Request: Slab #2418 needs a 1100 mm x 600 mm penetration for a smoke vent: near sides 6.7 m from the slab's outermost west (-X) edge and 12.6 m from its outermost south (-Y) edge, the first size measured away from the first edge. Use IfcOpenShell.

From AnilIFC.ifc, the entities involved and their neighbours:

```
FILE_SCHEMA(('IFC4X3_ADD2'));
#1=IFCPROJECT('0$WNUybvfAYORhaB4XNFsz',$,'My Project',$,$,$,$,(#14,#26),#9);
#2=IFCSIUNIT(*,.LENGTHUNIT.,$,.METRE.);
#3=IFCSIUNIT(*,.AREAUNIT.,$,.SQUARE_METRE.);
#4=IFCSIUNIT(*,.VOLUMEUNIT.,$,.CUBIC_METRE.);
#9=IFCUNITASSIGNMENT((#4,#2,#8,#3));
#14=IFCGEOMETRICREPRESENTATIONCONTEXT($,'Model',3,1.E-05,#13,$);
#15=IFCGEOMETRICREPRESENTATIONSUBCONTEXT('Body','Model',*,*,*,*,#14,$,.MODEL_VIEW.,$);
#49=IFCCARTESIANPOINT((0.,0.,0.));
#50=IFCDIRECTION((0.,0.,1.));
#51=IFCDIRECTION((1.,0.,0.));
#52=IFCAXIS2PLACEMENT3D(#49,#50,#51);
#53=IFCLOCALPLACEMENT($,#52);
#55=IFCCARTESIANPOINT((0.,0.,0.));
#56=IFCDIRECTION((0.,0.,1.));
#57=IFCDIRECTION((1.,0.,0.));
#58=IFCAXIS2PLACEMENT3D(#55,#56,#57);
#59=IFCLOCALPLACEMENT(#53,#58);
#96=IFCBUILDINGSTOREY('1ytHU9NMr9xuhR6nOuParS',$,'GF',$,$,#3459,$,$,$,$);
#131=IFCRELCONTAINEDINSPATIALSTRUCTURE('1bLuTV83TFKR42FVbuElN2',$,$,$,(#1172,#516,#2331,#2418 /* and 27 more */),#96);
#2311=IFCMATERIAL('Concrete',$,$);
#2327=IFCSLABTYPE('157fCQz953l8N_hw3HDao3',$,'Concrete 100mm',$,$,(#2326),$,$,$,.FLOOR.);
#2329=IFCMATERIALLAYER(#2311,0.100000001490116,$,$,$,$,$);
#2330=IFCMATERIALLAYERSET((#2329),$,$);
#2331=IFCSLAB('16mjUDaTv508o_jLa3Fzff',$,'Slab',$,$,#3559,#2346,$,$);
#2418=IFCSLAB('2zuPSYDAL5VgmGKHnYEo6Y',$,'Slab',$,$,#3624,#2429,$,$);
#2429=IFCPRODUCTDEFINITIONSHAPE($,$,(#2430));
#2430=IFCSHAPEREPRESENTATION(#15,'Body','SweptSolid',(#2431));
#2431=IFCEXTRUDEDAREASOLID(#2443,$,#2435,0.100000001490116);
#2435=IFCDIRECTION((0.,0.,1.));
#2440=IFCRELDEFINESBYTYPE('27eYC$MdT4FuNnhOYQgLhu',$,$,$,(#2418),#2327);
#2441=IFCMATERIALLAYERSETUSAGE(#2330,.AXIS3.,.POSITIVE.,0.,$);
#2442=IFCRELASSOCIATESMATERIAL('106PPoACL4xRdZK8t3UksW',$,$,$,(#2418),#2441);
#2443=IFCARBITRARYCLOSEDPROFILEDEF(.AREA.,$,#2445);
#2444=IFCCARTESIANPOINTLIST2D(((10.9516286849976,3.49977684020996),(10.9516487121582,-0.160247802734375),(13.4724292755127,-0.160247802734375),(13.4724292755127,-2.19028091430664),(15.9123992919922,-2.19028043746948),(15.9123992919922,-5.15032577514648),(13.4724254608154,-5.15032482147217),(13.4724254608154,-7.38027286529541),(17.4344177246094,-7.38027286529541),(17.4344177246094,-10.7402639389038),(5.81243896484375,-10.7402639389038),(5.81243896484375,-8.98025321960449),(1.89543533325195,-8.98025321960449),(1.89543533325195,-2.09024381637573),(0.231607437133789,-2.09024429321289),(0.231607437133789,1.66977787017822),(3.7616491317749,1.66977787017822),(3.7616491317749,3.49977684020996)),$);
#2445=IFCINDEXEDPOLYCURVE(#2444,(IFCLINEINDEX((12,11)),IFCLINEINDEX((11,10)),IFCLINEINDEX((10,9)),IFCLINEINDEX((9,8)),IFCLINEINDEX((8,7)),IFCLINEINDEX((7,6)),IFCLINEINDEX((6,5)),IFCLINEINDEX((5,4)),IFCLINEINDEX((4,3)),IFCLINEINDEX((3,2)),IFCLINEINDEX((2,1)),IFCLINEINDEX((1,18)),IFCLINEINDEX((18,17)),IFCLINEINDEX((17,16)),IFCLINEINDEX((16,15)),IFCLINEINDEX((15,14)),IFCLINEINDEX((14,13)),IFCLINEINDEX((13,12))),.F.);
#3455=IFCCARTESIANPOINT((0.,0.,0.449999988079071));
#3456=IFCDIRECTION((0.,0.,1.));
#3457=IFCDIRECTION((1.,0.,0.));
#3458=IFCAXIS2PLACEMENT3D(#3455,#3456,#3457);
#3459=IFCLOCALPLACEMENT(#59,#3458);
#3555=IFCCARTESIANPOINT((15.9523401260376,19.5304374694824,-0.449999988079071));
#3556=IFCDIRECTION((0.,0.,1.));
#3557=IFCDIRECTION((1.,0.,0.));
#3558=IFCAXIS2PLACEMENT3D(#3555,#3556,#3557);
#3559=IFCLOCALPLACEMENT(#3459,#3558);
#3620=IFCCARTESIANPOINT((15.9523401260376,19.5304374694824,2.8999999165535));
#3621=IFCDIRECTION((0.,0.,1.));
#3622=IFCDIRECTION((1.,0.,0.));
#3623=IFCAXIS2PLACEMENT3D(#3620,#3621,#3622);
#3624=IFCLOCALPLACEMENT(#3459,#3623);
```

```python
import numpy as np
import ifcopenshell
import ifcopenshell.api.feature
import ifcopenshell.api.geometry
import ifcopenshell.api.root
import ifcopenshell.geom
import ifcopenshell.util.placement
import ifcopenshell.util.representation
import ifcopenshell.util.shape
import ifcopenshell.util.unit

model = ifcopenshell.open("AnilIFC.ifc")
unit_scale = ifcopenshell.util.unit.calculate_unit_scale(model)
settings = ifcopenshell.geom.settings()


def volume(element):
    """Net volume in cubic metres, openings subtracted."""
    shape = ifcopenshell.geom.create_shape(settings, element)
    return ifcopenshell.util.shape.get_volume(shape.geometry)


slab = model.by_guid("2zuPSYDAL5VgmGKHnYEo6Y")
before = volume(slab)

# Extent in the slab's own axes, in metres. The edges named are its -X and -Y sides.
slab_shape = ifcopenshell.geom.create_shape(settings, slab)
vertices = ifcopenshell.util.shape.get_vertices(slab_shape.geometry)
x_min, y_min, bottom = vertices.min(axis=0)
top = vertices[:, 2].max()

opening = ifcopenshell.api.root.create_entity(model, ifc_class="IfcOpeningElement", name="Smoke vent opening", predefined_type="OPENING")
context = ifcopenshell.util.representation.get_context(model, "Model", "Body", "MODEL_VIEW")
width, depth = 1.1, 0.6
outline = [(0.0, 0.0), (width, 0.0), (width, depth), (0.0, depth), (0.0, 0.0)]
# Overshoot both faces by 50 mm so the cut is clean.
shape = ifcopenshell.api.geometry.add_slab_representation(
    model, context=context, depth=top - bottom + 0.1, polyline=outline
)
ifcopenshell.api.geometry.assign_representation(model, product=opening, representation=shape)

matrix = ifcopenshell.util.placement.get_local_placement(slab.ObjectPlacement)
matrix[:, 3] = matrix @ np.append(np.array([x_min + 6.7, y_min + 12.6, bottom - 0.05]) / unit_scale, 1.0)
ifcopenshell.api.geometry.edit_object_placement(model, product=opening, matrix=matrix, is_si=False)
ifcopenshell.api.feature.add_feature(model, feature=opening, element=slab)

after = volume(slab)

print(f"slab volume {before:.3f} -> {after:.3f} m3")

model.write("AnilIFC_edited.ifc")
```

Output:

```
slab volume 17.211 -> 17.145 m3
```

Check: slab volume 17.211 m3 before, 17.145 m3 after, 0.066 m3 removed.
